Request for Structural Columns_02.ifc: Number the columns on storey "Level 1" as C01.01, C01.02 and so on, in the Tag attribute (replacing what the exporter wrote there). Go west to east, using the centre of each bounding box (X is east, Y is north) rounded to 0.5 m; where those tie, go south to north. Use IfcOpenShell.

First a look at what the model holds.

```python
import ifcopenshell
import ifcopenshell.util.element
import ifcopenshell.util.placement

model = ifcopenshell.open("Structural Columns_02.ifc")
print(model.schema)
storey = next(s for s in model.by_type("IfcBuildingStorey") if s.Name == "Level 1")
columns = [e for e in ifcopenshell.util.element.get_decomposition(storey) if e.is_a("IfcColumn")]
for e in sorted(columns, key=lambda e: e.id()):
    origin = ifcopenshell.util.placement.get_local_placement(e.ObjectPlacement)[:3, 3]
    print(e.id(), e.Tag, e.Name, origin.round(2) + 0.0, sep=" | ")
```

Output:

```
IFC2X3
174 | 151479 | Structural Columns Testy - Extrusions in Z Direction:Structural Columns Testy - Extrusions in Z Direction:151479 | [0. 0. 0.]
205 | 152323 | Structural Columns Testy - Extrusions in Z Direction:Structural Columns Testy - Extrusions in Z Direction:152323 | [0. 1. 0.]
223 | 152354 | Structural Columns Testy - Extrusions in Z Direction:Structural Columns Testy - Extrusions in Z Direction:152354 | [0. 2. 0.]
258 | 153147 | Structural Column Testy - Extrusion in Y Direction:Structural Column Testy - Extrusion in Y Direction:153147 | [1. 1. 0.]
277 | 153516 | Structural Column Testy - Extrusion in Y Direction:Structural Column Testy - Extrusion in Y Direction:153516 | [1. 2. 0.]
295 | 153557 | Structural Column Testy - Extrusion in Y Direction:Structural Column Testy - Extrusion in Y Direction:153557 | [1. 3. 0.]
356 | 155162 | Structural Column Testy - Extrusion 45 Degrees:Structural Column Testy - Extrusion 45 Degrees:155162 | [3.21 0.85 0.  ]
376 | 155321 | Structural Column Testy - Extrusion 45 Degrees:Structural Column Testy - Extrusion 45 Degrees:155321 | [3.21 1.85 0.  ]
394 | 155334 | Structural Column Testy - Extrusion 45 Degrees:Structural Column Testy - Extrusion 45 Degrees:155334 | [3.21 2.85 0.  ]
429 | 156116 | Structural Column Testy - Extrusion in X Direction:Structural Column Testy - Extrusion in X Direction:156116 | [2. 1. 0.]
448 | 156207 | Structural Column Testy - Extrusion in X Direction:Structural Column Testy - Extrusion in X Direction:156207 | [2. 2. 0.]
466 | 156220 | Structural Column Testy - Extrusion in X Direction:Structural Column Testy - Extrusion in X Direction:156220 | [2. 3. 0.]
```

```python
import ifcopenshell
import ifcopenshell.geom
import ifcopenshell.util.element
import ifcopenshell.util.shape

model = ifcopenshell.open("Structural Columns_02.ifc")
settings = ifcopenshell.geom.settings()
settings.set("use-world-coords", True)


def centre(element):
    shape = ifcopenshell.geom.create_shape(settings, element)
    return ifcopenshell.util.shape.get_bbox_centroid(shape.geometry)


storey = next(s for s in model.by_type("IfcBuildingStorey") if s.Name == "Level 1")
columns = [e for e in ifcopenshell.util.element.get_decomposition(storey) if e.is_a("IfcColumn")]

# Insertion points can sit at a corner or the storey origin, so sort by the geometry (in metres).
centres = {e: centre(e) for e in columns}
columns.sort(key=lambda e: (round(centres[e][0] / 0.5), centres[e][1]))

for i, e in enumerate(columns, start=1):
    number = f"C01.{i:02d}"
    e.Tag = number
    print(e.id(), number)

model.write("Structural Columns_02_updated.ifc")
```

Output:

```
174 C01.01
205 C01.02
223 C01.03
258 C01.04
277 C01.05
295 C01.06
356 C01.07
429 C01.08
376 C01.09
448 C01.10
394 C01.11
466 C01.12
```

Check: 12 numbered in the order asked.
